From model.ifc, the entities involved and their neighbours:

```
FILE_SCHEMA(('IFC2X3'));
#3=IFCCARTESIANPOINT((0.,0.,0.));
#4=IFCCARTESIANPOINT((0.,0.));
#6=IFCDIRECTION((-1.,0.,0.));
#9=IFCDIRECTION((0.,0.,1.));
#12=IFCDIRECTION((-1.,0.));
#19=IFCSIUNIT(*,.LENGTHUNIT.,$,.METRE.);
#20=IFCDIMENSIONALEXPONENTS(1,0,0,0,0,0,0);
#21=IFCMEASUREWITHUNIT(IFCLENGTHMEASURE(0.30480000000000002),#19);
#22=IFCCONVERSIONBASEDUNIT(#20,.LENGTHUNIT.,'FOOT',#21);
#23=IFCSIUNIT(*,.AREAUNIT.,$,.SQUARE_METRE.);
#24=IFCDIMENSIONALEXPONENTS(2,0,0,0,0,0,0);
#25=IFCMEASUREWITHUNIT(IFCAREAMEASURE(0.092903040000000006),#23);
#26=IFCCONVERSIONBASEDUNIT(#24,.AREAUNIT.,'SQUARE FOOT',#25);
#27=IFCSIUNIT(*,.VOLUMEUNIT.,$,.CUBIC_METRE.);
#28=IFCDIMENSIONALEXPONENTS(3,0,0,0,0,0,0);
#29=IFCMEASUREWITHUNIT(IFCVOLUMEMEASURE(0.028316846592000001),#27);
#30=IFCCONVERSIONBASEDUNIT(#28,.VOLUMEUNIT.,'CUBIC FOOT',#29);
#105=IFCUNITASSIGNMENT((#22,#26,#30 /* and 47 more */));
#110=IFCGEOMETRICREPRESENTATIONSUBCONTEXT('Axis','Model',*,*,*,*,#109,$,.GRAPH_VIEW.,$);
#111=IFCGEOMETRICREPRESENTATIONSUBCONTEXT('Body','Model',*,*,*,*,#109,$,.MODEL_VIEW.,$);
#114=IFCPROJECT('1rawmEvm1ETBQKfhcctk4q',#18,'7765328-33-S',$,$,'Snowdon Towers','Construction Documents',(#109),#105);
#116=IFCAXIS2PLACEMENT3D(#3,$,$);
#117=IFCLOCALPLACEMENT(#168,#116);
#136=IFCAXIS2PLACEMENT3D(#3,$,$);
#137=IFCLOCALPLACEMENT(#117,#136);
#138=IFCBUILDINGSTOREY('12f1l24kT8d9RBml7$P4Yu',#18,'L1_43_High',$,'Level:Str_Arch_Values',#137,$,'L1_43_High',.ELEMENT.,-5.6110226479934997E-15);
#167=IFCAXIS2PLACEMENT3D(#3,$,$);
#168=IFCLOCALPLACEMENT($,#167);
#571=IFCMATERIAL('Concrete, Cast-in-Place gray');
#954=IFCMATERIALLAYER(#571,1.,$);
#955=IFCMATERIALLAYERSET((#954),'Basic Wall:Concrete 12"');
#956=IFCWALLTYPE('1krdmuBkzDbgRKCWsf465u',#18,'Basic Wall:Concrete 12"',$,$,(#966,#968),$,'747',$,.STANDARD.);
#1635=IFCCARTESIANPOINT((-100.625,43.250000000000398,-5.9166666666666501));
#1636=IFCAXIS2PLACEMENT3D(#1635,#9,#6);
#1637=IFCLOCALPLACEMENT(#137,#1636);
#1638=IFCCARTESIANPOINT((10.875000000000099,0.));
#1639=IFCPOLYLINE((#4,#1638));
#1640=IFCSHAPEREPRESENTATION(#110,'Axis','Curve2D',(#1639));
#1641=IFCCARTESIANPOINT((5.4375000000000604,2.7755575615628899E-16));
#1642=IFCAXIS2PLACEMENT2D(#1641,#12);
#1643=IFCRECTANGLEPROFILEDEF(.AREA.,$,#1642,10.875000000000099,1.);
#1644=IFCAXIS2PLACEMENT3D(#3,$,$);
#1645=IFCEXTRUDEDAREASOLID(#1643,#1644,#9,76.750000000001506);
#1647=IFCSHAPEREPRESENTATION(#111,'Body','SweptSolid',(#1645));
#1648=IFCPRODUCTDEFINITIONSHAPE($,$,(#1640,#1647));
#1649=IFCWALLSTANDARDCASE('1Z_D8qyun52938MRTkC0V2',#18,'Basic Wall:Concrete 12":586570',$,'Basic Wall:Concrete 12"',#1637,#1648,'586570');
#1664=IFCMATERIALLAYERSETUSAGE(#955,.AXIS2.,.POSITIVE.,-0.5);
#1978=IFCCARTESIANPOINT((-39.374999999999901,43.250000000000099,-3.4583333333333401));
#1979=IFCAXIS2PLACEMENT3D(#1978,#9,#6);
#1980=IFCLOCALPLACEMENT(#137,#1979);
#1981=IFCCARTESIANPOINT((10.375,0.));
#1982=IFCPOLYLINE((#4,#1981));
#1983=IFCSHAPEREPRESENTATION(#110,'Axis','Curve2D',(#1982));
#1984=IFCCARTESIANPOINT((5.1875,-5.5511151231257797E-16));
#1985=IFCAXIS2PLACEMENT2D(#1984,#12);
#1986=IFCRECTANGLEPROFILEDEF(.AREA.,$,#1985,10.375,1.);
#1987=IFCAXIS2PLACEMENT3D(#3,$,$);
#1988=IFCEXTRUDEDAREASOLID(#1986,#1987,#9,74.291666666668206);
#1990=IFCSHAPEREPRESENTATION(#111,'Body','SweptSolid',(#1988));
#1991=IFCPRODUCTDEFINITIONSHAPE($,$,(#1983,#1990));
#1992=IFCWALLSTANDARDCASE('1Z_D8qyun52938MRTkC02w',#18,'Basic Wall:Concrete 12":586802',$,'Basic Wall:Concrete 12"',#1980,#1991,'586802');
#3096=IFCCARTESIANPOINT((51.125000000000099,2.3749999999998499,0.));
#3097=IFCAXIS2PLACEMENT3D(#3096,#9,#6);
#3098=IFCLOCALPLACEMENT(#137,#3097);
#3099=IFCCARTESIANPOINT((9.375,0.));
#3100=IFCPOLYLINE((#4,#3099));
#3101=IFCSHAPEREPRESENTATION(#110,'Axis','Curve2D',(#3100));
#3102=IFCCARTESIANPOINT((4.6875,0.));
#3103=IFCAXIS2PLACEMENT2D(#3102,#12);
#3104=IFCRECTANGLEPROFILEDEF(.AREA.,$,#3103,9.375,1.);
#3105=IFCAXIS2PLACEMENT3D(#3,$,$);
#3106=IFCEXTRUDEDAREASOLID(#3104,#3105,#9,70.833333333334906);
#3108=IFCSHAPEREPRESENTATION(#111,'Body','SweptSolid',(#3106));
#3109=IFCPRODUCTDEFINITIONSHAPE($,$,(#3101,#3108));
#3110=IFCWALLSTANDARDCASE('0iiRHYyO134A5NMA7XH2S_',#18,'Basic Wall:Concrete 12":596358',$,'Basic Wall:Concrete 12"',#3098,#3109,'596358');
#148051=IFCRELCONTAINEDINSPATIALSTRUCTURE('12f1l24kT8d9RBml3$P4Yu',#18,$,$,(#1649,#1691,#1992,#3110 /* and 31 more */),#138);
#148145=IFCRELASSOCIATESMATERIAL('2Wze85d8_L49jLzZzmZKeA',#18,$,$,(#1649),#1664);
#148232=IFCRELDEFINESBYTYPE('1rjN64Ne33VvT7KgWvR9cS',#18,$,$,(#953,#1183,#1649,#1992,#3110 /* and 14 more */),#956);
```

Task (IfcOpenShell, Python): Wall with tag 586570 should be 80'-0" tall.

```python
import ifcopenshell
import ifcopenshell.geom
import ifcopenshell.util.representation
import ifcopenshell.util.shape
import ifcopenshell.util.unit

model = ifcopenshell.open("model.ifc")
unit_scale = ifcopenshell.util.unit.calculate_unit_scale(model)
settings = ifcopenshell.geom.settings()


def volume(element):
    """Net volume in cubic metres, openings subtracted."""
    shape = ifcopenshell.geom.create_shape(settings, element)
    return ifcopenshell.util.shape.get_volume(shape.geometry)


wall = model.by_id(1649)
before = volume(wall)

body = ifcopenshell.util.representation.get_representation(wall, "Model", "Body")
solid = body.Items[0]
old_height = solid.Depth
solid.Depth = 960 * 0.0254 / unit_scale
after = volume(wall)

print(f"height {old_height:g} -> {solid.Depth:g}, volume {before:.3f} -> {after:.3f} m3")

model.write("model_updated.ifc")
```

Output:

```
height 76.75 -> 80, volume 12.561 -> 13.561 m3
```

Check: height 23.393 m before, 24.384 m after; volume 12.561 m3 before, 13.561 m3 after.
